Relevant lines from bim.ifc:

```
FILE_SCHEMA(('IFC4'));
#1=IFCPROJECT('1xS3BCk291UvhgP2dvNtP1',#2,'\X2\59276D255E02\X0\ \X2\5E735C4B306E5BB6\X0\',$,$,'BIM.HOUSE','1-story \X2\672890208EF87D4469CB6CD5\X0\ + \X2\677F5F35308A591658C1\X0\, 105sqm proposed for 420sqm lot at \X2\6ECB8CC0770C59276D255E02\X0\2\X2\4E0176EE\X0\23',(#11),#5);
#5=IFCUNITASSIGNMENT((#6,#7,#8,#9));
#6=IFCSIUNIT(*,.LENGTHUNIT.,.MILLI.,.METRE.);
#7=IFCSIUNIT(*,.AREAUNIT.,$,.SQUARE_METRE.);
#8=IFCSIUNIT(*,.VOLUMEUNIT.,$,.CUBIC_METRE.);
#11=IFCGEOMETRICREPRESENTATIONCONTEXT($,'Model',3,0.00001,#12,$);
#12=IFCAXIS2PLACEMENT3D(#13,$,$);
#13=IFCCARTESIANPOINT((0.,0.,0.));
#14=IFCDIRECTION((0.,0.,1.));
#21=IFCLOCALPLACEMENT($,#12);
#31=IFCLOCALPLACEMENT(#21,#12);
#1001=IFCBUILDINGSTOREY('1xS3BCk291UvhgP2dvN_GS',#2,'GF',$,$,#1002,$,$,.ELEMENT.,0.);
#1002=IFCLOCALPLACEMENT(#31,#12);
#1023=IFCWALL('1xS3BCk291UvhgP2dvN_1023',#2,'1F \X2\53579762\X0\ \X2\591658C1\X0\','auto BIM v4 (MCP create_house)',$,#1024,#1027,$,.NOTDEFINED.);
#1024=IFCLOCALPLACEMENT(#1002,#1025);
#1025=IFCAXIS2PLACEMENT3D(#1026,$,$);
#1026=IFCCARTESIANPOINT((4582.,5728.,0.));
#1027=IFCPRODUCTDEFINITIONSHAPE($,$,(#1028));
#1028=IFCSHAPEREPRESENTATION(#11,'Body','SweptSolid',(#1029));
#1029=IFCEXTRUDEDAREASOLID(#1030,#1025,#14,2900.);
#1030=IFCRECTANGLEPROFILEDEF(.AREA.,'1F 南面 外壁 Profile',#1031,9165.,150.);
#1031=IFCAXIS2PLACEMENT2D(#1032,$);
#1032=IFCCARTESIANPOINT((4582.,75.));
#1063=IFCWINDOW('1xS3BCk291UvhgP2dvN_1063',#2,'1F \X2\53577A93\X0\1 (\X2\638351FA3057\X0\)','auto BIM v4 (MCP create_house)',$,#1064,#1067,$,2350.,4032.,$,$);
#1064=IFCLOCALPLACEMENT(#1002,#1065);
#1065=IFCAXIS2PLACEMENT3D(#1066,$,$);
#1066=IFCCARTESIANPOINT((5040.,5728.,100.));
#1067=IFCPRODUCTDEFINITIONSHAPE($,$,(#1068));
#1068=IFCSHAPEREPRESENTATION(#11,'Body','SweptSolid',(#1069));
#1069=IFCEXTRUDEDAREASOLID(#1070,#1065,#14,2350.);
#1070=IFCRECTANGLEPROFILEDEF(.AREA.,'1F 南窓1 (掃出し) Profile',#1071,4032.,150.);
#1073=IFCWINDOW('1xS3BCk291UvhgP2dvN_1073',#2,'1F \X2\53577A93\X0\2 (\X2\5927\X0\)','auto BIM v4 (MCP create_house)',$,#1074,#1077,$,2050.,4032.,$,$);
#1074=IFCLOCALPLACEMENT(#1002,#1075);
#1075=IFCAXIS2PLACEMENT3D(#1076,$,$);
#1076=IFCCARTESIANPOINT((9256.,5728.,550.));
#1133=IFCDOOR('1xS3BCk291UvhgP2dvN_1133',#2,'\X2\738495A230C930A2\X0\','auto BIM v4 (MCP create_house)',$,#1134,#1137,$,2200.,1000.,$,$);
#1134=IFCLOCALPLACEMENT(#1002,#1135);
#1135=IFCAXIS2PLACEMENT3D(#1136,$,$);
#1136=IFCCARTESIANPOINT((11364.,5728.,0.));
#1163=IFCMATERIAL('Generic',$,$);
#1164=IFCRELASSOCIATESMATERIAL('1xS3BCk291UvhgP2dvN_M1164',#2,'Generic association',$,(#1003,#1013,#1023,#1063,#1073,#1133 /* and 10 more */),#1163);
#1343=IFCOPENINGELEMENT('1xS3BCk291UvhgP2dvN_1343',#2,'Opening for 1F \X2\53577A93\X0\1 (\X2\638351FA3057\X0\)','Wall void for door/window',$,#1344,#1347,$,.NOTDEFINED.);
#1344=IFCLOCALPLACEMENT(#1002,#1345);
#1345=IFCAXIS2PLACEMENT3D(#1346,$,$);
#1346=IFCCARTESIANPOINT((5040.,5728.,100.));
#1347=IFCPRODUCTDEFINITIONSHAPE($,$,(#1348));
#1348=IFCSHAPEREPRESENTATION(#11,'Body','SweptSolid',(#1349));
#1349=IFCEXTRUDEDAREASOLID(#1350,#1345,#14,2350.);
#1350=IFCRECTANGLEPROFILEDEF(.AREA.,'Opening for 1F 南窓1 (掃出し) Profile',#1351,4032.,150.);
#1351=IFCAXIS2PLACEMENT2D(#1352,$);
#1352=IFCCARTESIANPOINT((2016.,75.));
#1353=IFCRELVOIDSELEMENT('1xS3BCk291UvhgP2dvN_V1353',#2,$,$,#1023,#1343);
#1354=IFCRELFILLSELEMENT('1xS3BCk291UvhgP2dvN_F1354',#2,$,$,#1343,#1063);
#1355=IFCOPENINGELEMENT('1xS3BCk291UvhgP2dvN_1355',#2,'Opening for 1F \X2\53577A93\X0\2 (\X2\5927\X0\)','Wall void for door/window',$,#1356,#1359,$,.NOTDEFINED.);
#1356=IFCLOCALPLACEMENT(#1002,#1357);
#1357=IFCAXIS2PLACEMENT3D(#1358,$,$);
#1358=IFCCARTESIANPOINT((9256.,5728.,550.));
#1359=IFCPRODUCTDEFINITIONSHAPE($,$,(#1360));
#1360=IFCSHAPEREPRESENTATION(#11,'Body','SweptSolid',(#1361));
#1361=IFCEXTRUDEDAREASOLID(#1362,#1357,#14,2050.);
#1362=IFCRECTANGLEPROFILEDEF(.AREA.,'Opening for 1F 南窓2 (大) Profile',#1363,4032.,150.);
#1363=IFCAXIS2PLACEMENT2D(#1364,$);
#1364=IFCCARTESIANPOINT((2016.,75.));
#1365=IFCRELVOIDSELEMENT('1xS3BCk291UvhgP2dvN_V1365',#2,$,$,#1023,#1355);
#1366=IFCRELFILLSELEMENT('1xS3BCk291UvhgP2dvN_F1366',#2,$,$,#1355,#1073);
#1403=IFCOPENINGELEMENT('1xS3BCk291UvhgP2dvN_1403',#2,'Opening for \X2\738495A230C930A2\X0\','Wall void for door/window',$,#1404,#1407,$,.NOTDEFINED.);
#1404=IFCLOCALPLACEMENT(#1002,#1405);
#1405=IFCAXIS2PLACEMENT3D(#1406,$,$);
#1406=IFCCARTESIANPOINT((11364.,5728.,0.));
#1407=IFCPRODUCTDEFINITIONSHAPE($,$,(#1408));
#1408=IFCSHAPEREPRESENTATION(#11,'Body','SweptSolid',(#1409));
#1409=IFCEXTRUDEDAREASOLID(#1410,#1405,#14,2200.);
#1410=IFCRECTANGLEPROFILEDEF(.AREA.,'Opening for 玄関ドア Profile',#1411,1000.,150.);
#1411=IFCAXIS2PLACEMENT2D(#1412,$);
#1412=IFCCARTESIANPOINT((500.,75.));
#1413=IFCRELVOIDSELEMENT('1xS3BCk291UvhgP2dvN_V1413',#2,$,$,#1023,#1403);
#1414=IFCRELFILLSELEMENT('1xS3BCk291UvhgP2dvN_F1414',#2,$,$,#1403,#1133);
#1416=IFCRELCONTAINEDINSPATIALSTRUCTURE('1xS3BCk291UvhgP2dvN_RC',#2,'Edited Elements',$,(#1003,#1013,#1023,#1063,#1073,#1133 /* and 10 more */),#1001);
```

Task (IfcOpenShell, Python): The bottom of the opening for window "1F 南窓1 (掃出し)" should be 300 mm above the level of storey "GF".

```python
import numpy as np
import ifcopenshell
import ifcopenshell.api.geometry
import ifcopenshell.geom
import ifcopenshell.util.element
import ifcopenshell.util.placement
import ifcopenshell.util.shape
import ifcopenshell.util.unit

model = ifcopenshell.open("bim.ifc")
unit_scale = ifcopenshell.util.unit.calculate_unit_scale(model)

window = model.by_guid("1xS3BCk291UvhgP2dvN_1063")
opening = window.FillsVoids[0].RelatingOpeningElement
storey = ifcopenshell.util.element.get_container(window, ifc_class="IfcBuildingStorey")
level = ifcopenshell.util.placement.get_local_placement(storey.ObjectPlacement)[2, 3]

# The opening's origin need not be at the sill, so measure its lowest point.
shape = ifcopenshell.geom.create_shape(ifcopenshell.geom.settings(), opening)
bottom = ifcopenshell.util.shape.get_shape_bottom_elevation(shape, shape.geometry) / unit_scale
dz = level + 0.3 / unit_scale - bottom

shift = np.array([0.0, 0.0, dz])
# The window is not placed relative to its opening, so move both.
for product in (opening, window):
    matrix = ifcopenshell.util.placement.get_local_placement(product.ObjectPlacement)
    matrix[:3, 3] += shift
    ifcopenshell.api.geometry.edit_object_placement(model, product=product, matrix=matrix, is_si=False)

print(f"moved by {dz * unit_scale:+.3f} m")

model.write("bim_v2.ifc")
```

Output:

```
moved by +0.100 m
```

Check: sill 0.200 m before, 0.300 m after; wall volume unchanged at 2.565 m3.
